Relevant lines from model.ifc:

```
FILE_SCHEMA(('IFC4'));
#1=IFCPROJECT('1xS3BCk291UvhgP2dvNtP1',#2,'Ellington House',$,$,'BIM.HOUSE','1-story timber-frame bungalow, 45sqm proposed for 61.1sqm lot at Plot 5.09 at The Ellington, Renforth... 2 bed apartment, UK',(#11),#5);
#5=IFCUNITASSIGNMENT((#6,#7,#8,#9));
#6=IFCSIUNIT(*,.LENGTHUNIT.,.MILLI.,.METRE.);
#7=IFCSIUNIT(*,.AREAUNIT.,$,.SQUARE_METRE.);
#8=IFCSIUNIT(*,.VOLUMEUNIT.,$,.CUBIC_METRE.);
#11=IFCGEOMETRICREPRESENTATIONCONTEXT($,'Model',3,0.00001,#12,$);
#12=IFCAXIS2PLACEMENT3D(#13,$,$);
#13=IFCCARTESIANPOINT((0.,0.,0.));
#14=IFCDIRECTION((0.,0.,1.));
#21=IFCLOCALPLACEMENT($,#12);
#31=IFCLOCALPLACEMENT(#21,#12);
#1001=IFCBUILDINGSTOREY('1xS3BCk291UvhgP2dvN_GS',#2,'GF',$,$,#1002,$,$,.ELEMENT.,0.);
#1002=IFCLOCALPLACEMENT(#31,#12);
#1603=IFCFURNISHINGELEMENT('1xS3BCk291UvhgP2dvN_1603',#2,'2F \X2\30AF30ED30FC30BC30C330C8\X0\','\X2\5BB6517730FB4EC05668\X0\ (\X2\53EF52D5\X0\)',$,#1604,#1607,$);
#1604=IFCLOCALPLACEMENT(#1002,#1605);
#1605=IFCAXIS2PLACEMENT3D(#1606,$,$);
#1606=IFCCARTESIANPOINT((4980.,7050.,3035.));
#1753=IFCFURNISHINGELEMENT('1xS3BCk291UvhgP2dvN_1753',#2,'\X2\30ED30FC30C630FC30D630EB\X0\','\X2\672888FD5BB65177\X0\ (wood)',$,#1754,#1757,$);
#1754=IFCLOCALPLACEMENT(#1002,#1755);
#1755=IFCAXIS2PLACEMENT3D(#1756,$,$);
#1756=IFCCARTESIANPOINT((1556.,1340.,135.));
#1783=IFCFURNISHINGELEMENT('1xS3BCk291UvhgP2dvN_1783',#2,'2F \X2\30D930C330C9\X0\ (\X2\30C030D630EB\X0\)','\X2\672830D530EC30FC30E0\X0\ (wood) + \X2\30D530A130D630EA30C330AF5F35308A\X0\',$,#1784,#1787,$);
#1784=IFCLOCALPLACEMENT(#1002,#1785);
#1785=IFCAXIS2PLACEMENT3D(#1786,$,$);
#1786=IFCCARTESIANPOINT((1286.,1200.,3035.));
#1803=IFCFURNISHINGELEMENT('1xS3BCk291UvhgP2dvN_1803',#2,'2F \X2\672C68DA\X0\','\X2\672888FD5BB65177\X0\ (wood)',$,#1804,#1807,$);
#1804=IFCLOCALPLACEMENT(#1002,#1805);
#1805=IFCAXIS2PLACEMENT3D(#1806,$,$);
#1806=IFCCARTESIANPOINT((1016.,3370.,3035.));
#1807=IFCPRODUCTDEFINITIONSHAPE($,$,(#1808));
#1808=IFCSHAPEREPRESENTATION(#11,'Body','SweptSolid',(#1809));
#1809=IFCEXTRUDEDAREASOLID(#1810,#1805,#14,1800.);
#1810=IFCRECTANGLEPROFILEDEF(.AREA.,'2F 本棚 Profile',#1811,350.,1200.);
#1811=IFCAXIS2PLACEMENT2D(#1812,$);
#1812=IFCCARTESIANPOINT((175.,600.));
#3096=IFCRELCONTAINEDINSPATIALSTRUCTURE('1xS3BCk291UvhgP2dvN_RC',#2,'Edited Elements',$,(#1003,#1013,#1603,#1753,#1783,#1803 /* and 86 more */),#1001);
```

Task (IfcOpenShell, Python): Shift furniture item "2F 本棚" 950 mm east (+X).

```python
import ifcopenshell
import ifcopenshell.api.geometry
import ifcopenshell.util.placement
import ifcopenshell.util.unit

model = ifcopenshell.open("model.ifc")
unit_scale = ifcopenshell.util.unit.calculate_unit_scale(model)

item = model.by_id(1803)
matrix = ifcopenshell.util.placement.get_local_placement(item.ObjectPlacement)
matrix[0, 3] += 0.95 / unit_scale
ifcopenshell.api.geometry.edit_object_placement(model, product=item, matrix=matrix, is_si=False)

print(ifcopenshell.util.placement.get_local_placement(item.ObjectPlacement).round(3) + 0.0)

model.write("model_v2.ifc")
```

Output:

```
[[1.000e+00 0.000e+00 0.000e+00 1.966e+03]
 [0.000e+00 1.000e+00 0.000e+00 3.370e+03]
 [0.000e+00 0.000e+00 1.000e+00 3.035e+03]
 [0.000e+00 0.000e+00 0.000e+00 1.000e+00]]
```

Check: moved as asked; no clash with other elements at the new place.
